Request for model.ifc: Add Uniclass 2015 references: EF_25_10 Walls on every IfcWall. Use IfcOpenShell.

First a look at what the model holds.

```python
import ifcopenshell

model = ifcopenshell.open("model.ifc")
print(model.schema)
print("classifications:", [c.Name for c in model.by_type("IfcClassification")])
for ifc_class in ("IfcDoor", "IfcRoof", "IfcStair", "IfcWall", "IfcWindow"):
    print(ifc_class, len(model.by_type(ifc_class)))
```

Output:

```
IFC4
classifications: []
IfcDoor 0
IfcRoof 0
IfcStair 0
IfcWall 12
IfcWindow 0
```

```python
import ifcopenshell
import ifcopenshell.api.classification

model = ifcopenshell.open("model.ifc")

system = ifcopenshell.api.classification.add_classification(model, classification="Uniclass 2015")

codes = {
    "IfcWall": ("EF_25_10", "Walls"),
}
for ifc_class, (code, name) in codes.items():
    products = model.by_type(ifc_class)
    ifcopenshell.api.classification.add_reference(
        model, products=products, classification=system, identification=code, name=name
    )
    print(code, len(products))

model.write("model_v2.ifc")
```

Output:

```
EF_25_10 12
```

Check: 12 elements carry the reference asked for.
